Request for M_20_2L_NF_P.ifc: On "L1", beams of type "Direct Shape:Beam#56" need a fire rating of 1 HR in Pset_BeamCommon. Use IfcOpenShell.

First a look at what the model holds.

```python
import ifcopenshell
import ifcopenshell.util.element

model = ifcopenshell.open("M_20_2L_NF_P.ifc")
print(model.schema)
storey = next(s for s in model.by_type("IfcBuildingStorey") if s.Name == "L1")
beams = [e for e in ifcopenshell.util.element.get_decomposition(storey) if e.is_a("IfcBeam")]
seen = {}
for e in beams:
    element_type = ifcopenshell.util.element.get_type(e)
    key = (element_type.Name if element_type != e and element_type else None, ifcopenshell.util.element.get_pset(e, "Pset_BeamCommon", "FireRating"))
    seen[key] = seen.get(key, 0) + 1
for (name, value), count in sorted(seen.items(), key=str):
    print(count, "x", name, "|", value)
```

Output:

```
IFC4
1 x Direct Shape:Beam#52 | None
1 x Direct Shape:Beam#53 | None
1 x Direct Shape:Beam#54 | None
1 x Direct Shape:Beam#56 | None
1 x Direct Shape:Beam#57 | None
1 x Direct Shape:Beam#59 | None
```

```python
import ifcopenshell
import ifcopenshell.api.pset
import ifcopenshell.util.element

model = ifcopenshell.open("M_20_2L_NF_P.ifc")

storey = next(s for s in model.by_type("IfcBuildingStorey") if s.Name == "L1")
beams = [e for e in ifcopenshell.util.element.get_decomposition(storey) if e.is_a("IfcBeam")]

count = 0
for e in beams:
    element_type = ifcopenshell.util.element.get_type(e)
    if element_type in (None, e) or element_type.Name != "Direct Shape:Beam#56":
        continue
    # add_pset returns the element's existing set when there is one.
    pset = ifcopenshell.api.pset.add_pset(model, product=e, name="Pset_BeamCommon")
    ifcopenshell.api.pset.edit_pset(model, pset=pset, properties={"FireRating": "1 HR"})
    count += 1

print(count, "beams updated")

model.write("M_20_2L_NF_P_rev.ifc")
```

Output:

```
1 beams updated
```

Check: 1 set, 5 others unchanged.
